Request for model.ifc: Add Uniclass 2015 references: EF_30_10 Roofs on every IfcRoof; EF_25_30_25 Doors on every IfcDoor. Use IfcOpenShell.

First a look at what the model holds.

```python
import ifcopenshell

model = ifcopenshell.open("model.ifc")
print(model.schema)
print("classifications:", [c.Name for c in model.by_type("IfcClassification")])
for ifc_class in ("IfcDoor", "IfcRoof", "IfcStair", "IfcWall", "IfcWindow"):
    print(ifc_class, len(model.by_type(ifc_class)))
```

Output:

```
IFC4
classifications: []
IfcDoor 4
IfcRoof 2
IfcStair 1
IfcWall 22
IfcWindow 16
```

```python
import ifcopenshell
import ifcopenshell.api.classification

model = ifcopenshell.open("model.ifc")

system = ifcopenshell.api.classification.add_classification(model, classification="Uniclass 2015")

codes = {
    "IfcRoof": ("EF_30_10", "Roofs"),
    "IfcDoor": ("EF_25_30_25", "Doors"),
}
for ifc_class, (code, name) in codes.items():
    products = model.by_type(ifc_class)
    ifcopenshell.api.classification.add_reference(
        model, products=products, classification=system, identification=code, name=name
    )
    print(code, len(products))

model.write("model-out.ifc")
```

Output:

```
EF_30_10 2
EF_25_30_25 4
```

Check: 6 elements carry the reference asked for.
